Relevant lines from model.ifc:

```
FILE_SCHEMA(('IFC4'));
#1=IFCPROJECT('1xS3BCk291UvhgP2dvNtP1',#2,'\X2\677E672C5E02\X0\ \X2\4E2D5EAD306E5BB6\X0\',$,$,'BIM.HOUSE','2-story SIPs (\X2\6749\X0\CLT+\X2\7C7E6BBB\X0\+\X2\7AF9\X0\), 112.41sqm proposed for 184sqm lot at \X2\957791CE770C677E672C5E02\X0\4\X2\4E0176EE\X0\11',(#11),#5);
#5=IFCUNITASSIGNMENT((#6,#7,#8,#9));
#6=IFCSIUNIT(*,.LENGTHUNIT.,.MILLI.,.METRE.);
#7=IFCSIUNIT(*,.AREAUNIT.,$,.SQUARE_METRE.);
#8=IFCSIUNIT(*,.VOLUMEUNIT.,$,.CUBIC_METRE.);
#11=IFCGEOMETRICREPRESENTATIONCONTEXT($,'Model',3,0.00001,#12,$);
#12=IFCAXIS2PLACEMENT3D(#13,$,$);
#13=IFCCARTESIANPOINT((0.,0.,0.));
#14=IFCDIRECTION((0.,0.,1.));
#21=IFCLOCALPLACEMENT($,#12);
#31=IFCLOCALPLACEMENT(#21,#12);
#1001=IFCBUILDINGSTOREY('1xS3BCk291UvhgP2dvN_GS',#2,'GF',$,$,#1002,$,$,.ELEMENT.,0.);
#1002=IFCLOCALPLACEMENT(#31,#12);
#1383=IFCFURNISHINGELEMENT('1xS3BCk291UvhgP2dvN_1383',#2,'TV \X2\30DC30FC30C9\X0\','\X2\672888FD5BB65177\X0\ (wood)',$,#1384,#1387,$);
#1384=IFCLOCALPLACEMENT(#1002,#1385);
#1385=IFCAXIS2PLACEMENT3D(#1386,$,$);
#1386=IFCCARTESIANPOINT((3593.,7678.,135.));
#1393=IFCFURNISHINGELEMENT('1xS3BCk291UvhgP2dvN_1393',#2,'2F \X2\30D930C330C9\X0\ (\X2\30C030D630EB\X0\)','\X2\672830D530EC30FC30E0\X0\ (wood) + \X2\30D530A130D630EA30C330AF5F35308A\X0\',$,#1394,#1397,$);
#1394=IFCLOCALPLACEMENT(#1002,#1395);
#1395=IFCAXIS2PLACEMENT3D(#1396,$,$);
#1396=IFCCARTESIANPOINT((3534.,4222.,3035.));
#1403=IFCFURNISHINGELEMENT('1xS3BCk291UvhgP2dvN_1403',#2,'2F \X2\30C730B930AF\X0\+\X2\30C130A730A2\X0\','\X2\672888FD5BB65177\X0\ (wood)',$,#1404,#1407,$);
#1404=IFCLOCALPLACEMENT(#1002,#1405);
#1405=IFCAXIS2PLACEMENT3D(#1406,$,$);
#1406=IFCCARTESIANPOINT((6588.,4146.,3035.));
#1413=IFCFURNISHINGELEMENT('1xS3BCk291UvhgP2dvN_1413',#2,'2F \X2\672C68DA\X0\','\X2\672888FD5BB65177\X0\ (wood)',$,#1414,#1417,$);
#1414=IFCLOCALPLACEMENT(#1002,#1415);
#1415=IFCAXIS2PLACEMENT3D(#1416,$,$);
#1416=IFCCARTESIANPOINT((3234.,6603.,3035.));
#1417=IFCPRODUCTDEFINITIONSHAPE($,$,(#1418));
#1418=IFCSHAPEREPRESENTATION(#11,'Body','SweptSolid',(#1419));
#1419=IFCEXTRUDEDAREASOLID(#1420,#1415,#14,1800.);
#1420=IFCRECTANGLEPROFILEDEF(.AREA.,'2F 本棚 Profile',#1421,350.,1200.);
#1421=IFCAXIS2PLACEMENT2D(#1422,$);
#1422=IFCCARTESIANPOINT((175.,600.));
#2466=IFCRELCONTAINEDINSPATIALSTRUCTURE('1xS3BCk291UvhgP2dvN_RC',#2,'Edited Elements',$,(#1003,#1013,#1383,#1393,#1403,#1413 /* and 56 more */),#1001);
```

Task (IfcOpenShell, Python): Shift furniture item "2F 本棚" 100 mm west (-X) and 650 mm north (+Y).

```python
import ifcopenshell
import ifcopenshell.api.geometry
import ifcopenshell.util.placement
import ifcopenshell.util.unit

model = ifcopenshell.open("model.ifc")
unit_scale = ifcopenshell.util.unit.calculate_unit_scale(model)

item = model.by_id(1413)
matrix = ifcopenshell.util.placement.get_local_placement(item.ObjectPlacement)
matrix[0, 3] -= 0.1 / unit_scale
matrix[1, 3] += 0.65 / unit_scale
ifcopenshell.api.geometry.edit_object_placement(model, product=item, matrix=matrix, is_si=False)

print(ifcopenshell.util.placement.get_local_placement(item.ObjectPlacement).round(3) + 0.0)

model.write("model_v2.ifc")
```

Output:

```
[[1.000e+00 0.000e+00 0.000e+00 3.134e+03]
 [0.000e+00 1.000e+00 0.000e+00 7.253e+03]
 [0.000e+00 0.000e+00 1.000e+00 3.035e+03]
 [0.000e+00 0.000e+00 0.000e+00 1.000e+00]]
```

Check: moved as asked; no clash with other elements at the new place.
